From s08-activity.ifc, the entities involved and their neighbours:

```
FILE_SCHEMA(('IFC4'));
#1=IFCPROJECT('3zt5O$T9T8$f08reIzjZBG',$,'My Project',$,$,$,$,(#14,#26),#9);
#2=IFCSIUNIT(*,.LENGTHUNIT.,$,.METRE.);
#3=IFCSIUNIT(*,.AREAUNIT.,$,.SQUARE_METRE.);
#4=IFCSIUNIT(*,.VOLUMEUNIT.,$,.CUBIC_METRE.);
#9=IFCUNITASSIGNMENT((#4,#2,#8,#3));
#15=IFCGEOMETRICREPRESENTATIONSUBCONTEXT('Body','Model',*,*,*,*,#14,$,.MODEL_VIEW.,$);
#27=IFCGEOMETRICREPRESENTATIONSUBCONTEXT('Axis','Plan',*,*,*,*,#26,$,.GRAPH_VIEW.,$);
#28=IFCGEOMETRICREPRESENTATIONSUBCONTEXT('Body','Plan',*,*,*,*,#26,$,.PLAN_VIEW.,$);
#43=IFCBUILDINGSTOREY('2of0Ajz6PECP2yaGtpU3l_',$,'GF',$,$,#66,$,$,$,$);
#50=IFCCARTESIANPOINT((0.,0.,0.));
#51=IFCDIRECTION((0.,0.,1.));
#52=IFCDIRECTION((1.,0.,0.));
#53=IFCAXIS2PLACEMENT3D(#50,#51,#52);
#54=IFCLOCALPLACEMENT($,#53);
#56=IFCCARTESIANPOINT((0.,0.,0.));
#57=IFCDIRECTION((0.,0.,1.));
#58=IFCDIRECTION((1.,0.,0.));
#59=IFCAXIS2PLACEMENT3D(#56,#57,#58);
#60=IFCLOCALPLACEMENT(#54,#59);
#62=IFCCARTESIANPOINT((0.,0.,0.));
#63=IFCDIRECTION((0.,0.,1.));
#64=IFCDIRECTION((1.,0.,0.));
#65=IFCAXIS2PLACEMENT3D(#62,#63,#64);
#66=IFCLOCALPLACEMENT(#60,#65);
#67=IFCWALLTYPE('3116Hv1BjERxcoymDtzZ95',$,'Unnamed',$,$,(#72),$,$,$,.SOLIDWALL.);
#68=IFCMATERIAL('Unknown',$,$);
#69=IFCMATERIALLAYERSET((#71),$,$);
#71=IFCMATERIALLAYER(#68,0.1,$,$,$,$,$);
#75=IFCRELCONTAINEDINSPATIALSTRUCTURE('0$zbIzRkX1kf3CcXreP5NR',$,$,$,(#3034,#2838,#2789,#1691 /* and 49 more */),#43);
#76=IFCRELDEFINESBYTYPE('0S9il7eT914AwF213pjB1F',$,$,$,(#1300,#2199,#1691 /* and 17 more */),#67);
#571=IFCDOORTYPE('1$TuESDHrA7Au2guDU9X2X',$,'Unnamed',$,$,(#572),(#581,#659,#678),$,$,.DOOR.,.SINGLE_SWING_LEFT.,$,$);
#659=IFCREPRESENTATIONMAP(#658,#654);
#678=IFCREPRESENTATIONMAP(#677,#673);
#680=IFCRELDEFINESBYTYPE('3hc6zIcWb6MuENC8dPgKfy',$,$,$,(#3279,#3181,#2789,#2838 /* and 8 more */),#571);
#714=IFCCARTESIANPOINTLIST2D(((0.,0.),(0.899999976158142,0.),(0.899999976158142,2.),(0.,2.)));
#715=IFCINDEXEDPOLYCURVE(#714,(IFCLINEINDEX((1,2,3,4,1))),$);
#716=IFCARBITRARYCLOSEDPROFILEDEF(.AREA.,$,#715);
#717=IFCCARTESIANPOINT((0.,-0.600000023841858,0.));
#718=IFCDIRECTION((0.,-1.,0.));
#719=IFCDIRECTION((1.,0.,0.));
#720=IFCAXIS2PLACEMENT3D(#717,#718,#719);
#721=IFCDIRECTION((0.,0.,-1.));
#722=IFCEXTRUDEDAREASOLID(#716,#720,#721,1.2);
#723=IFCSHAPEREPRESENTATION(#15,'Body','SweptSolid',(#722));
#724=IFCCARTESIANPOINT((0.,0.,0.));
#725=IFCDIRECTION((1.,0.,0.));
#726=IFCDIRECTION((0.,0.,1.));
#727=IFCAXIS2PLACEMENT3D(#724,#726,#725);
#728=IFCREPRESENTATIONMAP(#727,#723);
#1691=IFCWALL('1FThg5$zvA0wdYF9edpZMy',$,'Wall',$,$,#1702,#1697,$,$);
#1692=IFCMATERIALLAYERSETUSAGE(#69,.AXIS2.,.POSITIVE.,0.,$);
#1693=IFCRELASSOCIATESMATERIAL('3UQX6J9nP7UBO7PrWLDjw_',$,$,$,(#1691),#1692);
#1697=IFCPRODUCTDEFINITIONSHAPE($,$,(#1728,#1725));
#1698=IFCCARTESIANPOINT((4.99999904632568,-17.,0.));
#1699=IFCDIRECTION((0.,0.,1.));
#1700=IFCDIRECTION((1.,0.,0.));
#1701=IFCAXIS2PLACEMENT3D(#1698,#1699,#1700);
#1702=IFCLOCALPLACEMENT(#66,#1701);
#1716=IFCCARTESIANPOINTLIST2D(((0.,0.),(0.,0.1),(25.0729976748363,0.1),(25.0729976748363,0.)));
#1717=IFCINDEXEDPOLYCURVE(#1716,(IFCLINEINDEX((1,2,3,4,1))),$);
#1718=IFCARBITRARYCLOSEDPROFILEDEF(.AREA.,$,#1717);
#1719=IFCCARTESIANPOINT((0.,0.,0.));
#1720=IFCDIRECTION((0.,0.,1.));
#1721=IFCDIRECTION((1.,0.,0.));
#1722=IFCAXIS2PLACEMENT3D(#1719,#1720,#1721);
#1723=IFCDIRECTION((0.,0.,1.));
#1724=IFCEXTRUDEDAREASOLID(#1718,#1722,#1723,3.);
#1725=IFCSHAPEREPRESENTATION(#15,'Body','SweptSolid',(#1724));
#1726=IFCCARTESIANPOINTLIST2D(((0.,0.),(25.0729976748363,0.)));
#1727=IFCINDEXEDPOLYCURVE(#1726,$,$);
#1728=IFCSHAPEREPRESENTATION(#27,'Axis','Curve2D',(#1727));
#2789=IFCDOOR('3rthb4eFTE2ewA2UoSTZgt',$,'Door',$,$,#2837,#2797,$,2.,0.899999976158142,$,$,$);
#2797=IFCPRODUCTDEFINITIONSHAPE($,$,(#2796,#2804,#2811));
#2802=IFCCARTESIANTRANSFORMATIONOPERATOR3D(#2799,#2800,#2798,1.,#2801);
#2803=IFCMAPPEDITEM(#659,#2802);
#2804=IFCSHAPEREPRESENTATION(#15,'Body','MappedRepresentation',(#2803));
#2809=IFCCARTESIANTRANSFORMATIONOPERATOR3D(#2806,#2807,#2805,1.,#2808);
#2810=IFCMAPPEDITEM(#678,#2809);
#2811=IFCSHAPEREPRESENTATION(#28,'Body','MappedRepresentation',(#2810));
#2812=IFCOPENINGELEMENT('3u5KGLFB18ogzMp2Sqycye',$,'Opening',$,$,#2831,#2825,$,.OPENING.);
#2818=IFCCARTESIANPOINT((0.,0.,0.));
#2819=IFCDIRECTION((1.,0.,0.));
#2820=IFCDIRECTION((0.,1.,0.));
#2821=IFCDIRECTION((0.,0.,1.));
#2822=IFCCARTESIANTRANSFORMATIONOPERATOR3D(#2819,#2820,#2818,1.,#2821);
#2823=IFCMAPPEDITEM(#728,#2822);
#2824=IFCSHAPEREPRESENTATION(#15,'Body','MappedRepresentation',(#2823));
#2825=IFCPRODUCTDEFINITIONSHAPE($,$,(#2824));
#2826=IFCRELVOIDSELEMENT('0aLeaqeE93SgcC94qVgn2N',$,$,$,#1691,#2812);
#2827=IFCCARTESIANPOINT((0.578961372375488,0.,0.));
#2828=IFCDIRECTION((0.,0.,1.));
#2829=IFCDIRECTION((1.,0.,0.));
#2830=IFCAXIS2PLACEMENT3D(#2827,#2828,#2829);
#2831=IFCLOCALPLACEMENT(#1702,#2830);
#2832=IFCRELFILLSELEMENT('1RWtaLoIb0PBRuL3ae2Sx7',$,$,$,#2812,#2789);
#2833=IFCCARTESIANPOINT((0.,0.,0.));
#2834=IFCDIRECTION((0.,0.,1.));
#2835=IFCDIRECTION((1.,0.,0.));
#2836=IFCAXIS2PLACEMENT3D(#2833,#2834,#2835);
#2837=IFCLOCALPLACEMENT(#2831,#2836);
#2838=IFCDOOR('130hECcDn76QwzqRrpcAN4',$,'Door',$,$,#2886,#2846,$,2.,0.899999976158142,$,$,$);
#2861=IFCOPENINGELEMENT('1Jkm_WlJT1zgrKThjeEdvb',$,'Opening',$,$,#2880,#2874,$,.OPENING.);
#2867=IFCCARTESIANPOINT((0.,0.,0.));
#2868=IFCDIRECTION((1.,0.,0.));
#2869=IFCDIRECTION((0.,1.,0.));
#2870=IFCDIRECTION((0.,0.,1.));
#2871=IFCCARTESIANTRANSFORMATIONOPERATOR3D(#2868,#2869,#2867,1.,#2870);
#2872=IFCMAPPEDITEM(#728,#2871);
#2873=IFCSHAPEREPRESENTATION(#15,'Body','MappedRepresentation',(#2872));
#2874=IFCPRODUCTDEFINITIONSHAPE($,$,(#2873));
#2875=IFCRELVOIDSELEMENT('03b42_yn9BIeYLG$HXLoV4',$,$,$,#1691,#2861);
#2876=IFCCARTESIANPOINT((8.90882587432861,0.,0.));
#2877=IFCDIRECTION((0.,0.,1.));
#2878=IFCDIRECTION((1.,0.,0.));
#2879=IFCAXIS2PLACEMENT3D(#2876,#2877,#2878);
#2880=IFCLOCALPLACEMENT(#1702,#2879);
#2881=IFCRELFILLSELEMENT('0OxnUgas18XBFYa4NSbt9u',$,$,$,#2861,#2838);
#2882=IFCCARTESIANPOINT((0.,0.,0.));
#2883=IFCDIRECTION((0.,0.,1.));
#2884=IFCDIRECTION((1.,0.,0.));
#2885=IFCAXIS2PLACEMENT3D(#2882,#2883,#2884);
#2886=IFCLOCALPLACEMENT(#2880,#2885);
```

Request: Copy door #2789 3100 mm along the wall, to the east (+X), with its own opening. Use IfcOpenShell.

```python
import ifcopenshell
import ifcopenshell.api.feature
import ifcopenshell.api.geometry
import ifcopenshell.api.root
import ifcopenshell.geom
import ifcopenshell.util.element
import ifcopenshell.util.placement
import ifcopenshell.util.shape
import ifcopenshell.util.unit

model = ifcopenshell.open("s08-activity.ifc")
unit_scale = ifcopenshell.util.unit.calculate_unit_scale(model)
settings = ifcopenshell.geom.settings()


def volume(element):
    """Net volume in cubic metres, openings subtracted."""
    shape = ifcopenshell.geom.create_shape(settings, element)
    return ifcopenshell.util.shape.get_volume(shape.geometry)


door = model.by_guid("3rthb4eFTE2ewA2UoSTZgt")
opening = door.FillsVoids[0].RelatingOpeningElement
wall = opening.VoidsElements[0].RelatingBuildingElement
before = volume(wall)
shift = ifcopenshell.util.placement.get_local_placement(wall.ObjectPlacement)[:3, 0] * 3.1 / unit_scale

# copy_class copies the void relationship, type, container and properties, but no geometry.
new_opening = ifcopenshell.api.root.copy_class(model, product=opening)
new_opening.Representation = ifcopenshell.util.element.copy_deep(
    model, opening.Representation, exclude=["IfcGeometricRepresentationContext", "IfcRepresentationMap"]
)
new_door = ifcopenshell.api.root.copy_class(model, product=door)
new_door.Representation = ifcopenshell.util.element.copy_deep(
    model, door.Representation, exclude=["IfcGeometricRepresentationContext", "IfcRepresentationMap"]
)
ifcopenshell.api.feature.add_filling(model, opening=new_opening, element=new_door)

for old, new in ((opening, new_opening), (door, new_door)):
    matrix = ifcopenshell.util.placement.get_local_placement(old.ObjectPlacement)
    matrix[:3, 3] += shift
    ifcopenshell.api.geometry.edit_object_placement(model, product=new, matrix=matrix, is_si=False)

after = volume(wall)

print(f"wall volume {before:.3f} -> {after:.3f} m3")

model.write("s08-activity_rev.ifc")
```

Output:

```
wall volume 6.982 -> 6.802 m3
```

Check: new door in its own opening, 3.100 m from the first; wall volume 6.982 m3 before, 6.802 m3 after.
